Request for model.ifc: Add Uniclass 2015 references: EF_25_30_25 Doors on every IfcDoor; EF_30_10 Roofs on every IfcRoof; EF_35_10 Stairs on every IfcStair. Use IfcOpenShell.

First a look at what the model holds.

```python
import ifcopenshell

model = ifcopenshell.open("model.ifc")
print(model.schema)
print("classifications:", [c.Name for c in model.by_type("IfcClassification")])
for ifc_class in ("IfcDoor", "IfcRoof", "IfcStair", "IfcWall", "IfcWindow"):
    print(ifc_class, len(model.by_type(ifc_class)))
```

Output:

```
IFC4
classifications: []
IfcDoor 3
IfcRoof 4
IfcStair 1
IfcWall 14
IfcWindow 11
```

```python
import ifcopenshell
import ifcopenshell.api.classification

model = ifcopenshell.open("model.ifc")

system = ifcopenshell.api.classification.add_classification(model, classification="Uniclass 2015")

codes = {
    "IfcDoor": ("EF_25_30_25", "Doors"),
    "IfcRoof": ("EF_30_10", "Roofs"),
    "IfcStair": ("EF_35_10", "Stairs"),
}
for ifc_class, (code, name) in codes.items():
    products = model.by_type(ifc_class)
    ifcopenshell.api.classification.add_reference(
        model, products=products, classification=system, identification=code, name=name
    )
    print(code, len(products))

model.write("model-out.ifc")
```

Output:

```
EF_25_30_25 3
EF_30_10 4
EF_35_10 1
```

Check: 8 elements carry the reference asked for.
